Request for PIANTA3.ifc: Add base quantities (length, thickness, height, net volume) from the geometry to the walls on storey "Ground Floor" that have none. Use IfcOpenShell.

First a look at what the model holds.

```python
import ifcopenshell
import ifcopenshell.util.element
import ifcopenshell.util.unit

model = ifcopenshell.open("PIANTA3.ifc")
print(model.schema)
for unit_type in ("LENGTHUNIT", "AREAUNIT", "VOLUMEUNIT"):
    print(unit_type, ifcopenshell.util.unit.calculate_unit_scale(model, unit_type))
storey = next(s for s in model.by_type("IfcBuildingStorey") if s.Name == "Ground Floor")
walls = [e for e in ifcopenshell.util.element.get_decomposition(storey) if e.is_a("IfcWall")]
for e in sorted(walls, key=lambda e: e.id()):
    print(e.id(), e.is_a(), e.Name, list(ifcopenshell.util.element.get_psets(e, qtos_only=True)), sep=" | ")
```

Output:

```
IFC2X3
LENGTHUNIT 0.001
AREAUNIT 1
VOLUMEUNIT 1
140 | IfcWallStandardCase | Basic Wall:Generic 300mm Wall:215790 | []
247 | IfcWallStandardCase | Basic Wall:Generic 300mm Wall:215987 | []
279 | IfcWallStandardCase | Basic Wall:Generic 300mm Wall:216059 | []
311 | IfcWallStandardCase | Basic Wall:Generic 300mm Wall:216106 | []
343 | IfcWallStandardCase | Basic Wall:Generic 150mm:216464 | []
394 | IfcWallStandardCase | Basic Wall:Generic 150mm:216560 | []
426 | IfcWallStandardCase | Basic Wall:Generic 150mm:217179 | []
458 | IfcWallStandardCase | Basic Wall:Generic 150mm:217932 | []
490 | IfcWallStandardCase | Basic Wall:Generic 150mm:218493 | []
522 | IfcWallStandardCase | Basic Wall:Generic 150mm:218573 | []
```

```python
import ifcopenshell
import ifcopenshell.api.pset
import ifcopenshell.geom
import ifcopenshell.util.element
import ifcopenshell.util.shape
import ifcopenshell.util.unit

model = ifcopenshell.open("PIANTA3.ifc")
unit_scale = ifcopenshell.util.unit.calculate_unit_scale(model)
volume_scale = ifcopenshell.util.unit.calculate_unit_scale(model, "VOLUMEUNIT")
settings = ifcopenshell.geom.settings()

storey = next(s for s in model.by_type("IfcBuildingStorey") if s.Name == "Ground Floor")
walls = [e for e in ifcopenshell.util.element.get_decomposition(storey) if e.is_a("IfcWall")]

for e in sorted(walls, key=lambda e: e.id()):
    if ifcopenshell.util.element.get_psets(e, qtos_only=True, should_inherit=False):
        continue
    # Geometry comes back in metres, in the element's own axes.
    shape = ifcopenshell.geom.create_shape(settings, e)
    values = {
        "Length": ifcopenshell.util.shape.get_x(shape.geometry) / unit_scale,
        "Width": ifcopenshell.util.shape.get_y(shape.geometry) / unit_scale,
        "Height": ifcopenshell.util.shape.get_z(shape.geometry) / unit_scale,
        "NetVolume": ifcopenshell.util.shape.get_volume(shape.geometry) / volume_scale,
    }
    qto = ifcopenshell.api.pset.add_qto(model, product=e, name="BaseQuantities")
    ifcopenshell.api.pset.edit_qto(model, qto=qto, properties=values)
    print(e.id(), {k: round(v, 3) for k, v in values.items()})

model.write("PIANTA3_v2.ifc")
```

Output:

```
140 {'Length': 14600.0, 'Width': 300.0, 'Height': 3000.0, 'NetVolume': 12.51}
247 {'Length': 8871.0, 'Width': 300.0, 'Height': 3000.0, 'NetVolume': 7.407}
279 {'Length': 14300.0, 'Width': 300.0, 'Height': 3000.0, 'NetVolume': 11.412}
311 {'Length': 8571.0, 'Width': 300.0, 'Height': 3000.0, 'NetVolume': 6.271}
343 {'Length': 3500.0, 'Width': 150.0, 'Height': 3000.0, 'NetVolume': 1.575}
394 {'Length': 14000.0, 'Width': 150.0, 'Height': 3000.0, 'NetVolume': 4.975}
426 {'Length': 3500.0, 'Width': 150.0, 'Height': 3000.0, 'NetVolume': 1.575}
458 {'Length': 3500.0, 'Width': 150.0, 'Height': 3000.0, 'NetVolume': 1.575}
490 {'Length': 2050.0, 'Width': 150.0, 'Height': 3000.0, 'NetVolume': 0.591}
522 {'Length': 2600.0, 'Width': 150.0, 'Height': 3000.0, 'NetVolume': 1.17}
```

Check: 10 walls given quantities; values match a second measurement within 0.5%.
